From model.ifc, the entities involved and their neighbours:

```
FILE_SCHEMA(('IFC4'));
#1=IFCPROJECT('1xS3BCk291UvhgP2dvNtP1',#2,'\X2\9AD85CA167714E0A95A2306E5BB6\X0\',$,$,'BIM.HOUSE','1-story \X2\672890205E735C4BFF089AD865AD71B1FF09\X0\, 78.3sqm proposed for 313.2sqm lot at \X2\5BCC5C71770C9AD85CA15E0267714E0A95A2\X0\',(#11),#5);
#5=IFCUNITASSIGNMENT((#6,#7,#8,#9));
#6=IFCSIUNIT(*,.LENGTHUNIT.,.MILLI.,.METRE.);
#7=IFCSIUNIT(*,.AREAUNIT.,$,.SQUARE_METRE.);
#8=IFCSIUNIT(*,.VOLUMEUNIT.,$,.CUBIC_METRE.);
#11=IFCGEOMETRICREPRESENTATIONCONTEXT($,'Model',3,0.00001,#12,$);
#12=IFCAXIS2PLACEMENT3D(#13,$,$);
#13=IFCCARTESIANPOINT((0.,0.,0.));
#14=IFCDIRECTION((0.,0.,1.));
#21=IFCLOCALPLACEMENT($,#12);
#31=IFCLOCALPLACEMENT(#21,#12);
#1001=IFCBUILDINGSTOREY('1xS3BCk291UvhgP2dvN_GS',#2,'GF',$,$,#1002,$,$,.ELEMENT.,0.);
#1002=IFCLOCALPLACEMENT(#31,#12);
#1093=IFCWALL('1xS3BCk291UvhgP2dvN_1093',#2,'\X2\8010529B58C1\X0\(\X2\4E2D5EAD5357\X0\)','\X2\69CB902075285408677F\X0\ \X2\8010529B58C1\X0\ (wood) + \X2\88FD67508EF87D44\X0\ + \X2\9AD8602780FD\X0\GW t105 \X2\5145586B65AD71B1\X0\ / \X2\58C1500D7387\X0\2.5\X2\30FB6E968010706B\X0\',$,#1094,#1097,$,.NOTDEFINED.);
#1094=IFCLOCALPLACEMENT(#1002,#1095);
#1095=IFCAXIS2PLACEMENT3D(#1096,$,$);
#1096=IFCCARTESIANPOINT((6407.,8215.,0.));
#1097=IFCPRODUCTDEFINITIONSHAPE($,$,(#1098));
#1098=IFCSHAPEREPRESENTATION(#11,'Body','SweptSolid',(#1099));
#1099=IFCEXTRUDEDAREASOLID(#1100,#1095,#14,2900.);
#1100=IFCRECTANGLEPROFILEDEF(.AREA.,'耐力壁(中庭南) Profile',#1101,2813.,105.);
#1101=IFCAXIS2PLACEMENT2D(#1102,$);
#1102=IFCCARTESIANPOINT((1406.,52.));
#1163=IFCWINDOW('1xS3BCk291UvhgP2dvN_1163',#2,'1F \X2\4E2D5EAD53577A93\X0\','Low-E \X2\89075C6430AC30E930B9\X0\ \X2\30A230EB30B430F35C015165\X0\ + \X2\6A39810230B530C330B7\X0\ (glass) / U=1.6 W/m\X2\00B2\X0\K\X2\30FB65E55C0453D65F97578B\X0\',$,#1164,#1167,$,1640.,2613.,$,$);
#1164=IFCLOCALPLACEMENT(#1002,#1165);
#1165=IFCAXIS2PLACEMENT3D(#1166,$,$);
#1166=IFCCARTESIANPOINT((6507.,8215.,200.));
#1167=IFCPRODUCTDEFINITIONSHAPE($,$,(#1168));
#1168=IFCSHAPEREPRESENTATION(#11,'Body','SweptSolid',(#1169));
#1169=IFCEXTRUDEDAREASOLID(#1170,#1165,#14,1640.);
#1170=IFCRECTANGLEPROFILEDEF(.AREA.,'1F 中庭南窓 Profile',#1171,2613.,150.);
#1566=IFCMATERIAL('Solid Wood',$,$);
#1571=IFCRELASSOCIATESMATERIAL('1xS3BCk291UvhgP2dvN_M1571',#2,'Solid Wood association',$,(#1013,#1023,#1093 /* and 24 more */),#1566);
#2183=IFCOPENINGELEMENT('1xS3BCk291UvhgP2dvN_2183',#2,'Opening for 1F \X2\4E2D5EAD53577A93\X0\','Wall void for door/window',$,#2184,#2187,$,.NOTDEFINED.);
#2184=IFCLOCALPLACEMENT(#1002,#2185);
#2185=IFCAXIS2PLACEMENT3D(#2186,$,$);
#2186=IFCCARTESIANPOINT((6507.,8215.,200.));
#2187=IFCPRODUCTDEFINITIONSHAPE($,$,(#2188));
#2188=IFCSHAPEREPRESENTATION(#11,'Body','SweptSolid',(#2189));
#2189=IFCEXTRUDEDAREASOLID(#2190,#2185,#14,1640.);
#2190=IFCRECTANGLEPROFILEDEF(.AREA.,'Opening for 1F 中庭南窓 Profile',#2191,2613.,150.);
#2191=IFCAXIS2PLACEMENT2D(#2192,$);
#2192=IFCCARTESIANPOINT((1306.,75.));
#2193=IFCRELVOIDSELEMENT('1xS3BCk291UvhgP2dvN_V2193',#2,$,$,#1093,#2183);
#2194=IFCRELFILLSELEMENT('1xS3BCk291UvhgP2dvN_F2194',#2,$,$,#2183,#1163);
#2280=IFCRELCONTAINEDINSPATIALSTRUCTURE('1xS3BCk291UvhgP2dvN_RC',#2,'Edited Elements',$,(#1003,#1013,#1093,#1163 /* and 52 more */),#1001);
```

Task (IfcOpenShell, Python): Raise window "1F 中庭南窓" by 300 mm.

```python
import numpy as np
import ifcopenshell
import ifcopenshell.api.geometry
import ifcopenshell.util.placement
import ifcopenshell.util.unit

model = ifcopenshell.open("model.ifc")
unit_scale = ifcopenshell.util.unit.calculate_unit_scale(model)

window = model.by_guid("1xS3BCk291UvhgP2dvN_1163")
opening = window.FillsVoids[0].RelatingOpeningElement
dz = 300.0

shift = np.array([0.0, 0.0, dz])
# The window is not placed relative to its opening, so move both.
for product in (opening, window):
    matrix = ifcopenshell.util.placement.get_local_placement(product.ObjectPlacement)
    matrix[:3, 3] += shift
    ifcopenshell.api.geometry.edit_object_placement(model, product=product, matrix=matrix, is_si=False)

print(f"moved by {dz * unit_scale:+.3f} m")

model.write("model_edited.ifc")
```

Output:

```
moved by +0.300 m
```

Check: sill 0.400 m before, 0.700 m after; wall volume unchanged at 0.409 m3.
